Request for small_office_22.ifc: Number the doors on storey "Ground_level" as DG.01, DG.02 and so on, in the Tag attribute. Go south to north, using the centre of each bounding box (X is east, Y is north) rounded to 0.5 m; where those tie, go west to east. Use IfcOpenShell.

First a look at what the model holds.

```python
import ifcopenshell
import ifcopenshell.util.element
import ifcopenshell.util.placement

model = ifcopenshell.open("small_office_22.ifc")
print(model.schema)
storey = next(s for s in model.by_type("IfcBuildingStorey") if s.Name == "Ground_level")
doors = [e for e in ifcopenshell.util.element.get_decomposition(storey) if e.is_a("IfcDoor")]
for e in sorted(doors, key=lambda e: e.id()):
    origin = ifcopenshell.util.placement.get_local_placement(e.ObjectPlacement)[:3, 3]
    print(e.id(), e.Tag, e.Name, origin.round(2) + 0.0, sep=" | ")
```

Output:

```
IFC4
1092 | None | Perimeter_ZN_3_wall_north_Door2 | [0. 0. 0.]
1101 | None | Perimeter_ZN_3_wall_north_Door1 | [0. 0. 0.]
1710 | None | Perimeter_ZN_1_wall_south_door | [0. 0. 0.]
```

```python
import ifcopenshell
import ifcopenshell.geom
import ifcopenshell.util.element
import ifcopenshell.util.shape

model = ifcopenshell.open("small_office_22.ifc")
settings = ifcopenshell.geom.settings()
settings.set("use-world-coords", True)


def centre(element):
    shape = ifcopenshell.geom.create_shape(settings, element)
    return ifcopenshell.util.shape.get_bbox_centroid(shape.geometry)


storey = next(s for s in model.by_type("IfcBuildingStorey") if s.Name == "Ground_level")
doors = [e for e in ifcopenshell.util.element.get_decomposition(storey) if e.is_a("IfcDoor")]

# Insertion points can sit at a corner or the storey origin, so sort by the geometry (in metres).
centres = {e: centre(e) for e in doors}
doors.sort(key=lambda e: (round(centres[e][1] / 0.5), centres[e][0]))

for i, e in enumerate(doors, start=1):
    number = f"DG.{i:02d}"
    e.Tag = number
    print(e.id(), number)

model.write("small_office_22_rev.ifc")
```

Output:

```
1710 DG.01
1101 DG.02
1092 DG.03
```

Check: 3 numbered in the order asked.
